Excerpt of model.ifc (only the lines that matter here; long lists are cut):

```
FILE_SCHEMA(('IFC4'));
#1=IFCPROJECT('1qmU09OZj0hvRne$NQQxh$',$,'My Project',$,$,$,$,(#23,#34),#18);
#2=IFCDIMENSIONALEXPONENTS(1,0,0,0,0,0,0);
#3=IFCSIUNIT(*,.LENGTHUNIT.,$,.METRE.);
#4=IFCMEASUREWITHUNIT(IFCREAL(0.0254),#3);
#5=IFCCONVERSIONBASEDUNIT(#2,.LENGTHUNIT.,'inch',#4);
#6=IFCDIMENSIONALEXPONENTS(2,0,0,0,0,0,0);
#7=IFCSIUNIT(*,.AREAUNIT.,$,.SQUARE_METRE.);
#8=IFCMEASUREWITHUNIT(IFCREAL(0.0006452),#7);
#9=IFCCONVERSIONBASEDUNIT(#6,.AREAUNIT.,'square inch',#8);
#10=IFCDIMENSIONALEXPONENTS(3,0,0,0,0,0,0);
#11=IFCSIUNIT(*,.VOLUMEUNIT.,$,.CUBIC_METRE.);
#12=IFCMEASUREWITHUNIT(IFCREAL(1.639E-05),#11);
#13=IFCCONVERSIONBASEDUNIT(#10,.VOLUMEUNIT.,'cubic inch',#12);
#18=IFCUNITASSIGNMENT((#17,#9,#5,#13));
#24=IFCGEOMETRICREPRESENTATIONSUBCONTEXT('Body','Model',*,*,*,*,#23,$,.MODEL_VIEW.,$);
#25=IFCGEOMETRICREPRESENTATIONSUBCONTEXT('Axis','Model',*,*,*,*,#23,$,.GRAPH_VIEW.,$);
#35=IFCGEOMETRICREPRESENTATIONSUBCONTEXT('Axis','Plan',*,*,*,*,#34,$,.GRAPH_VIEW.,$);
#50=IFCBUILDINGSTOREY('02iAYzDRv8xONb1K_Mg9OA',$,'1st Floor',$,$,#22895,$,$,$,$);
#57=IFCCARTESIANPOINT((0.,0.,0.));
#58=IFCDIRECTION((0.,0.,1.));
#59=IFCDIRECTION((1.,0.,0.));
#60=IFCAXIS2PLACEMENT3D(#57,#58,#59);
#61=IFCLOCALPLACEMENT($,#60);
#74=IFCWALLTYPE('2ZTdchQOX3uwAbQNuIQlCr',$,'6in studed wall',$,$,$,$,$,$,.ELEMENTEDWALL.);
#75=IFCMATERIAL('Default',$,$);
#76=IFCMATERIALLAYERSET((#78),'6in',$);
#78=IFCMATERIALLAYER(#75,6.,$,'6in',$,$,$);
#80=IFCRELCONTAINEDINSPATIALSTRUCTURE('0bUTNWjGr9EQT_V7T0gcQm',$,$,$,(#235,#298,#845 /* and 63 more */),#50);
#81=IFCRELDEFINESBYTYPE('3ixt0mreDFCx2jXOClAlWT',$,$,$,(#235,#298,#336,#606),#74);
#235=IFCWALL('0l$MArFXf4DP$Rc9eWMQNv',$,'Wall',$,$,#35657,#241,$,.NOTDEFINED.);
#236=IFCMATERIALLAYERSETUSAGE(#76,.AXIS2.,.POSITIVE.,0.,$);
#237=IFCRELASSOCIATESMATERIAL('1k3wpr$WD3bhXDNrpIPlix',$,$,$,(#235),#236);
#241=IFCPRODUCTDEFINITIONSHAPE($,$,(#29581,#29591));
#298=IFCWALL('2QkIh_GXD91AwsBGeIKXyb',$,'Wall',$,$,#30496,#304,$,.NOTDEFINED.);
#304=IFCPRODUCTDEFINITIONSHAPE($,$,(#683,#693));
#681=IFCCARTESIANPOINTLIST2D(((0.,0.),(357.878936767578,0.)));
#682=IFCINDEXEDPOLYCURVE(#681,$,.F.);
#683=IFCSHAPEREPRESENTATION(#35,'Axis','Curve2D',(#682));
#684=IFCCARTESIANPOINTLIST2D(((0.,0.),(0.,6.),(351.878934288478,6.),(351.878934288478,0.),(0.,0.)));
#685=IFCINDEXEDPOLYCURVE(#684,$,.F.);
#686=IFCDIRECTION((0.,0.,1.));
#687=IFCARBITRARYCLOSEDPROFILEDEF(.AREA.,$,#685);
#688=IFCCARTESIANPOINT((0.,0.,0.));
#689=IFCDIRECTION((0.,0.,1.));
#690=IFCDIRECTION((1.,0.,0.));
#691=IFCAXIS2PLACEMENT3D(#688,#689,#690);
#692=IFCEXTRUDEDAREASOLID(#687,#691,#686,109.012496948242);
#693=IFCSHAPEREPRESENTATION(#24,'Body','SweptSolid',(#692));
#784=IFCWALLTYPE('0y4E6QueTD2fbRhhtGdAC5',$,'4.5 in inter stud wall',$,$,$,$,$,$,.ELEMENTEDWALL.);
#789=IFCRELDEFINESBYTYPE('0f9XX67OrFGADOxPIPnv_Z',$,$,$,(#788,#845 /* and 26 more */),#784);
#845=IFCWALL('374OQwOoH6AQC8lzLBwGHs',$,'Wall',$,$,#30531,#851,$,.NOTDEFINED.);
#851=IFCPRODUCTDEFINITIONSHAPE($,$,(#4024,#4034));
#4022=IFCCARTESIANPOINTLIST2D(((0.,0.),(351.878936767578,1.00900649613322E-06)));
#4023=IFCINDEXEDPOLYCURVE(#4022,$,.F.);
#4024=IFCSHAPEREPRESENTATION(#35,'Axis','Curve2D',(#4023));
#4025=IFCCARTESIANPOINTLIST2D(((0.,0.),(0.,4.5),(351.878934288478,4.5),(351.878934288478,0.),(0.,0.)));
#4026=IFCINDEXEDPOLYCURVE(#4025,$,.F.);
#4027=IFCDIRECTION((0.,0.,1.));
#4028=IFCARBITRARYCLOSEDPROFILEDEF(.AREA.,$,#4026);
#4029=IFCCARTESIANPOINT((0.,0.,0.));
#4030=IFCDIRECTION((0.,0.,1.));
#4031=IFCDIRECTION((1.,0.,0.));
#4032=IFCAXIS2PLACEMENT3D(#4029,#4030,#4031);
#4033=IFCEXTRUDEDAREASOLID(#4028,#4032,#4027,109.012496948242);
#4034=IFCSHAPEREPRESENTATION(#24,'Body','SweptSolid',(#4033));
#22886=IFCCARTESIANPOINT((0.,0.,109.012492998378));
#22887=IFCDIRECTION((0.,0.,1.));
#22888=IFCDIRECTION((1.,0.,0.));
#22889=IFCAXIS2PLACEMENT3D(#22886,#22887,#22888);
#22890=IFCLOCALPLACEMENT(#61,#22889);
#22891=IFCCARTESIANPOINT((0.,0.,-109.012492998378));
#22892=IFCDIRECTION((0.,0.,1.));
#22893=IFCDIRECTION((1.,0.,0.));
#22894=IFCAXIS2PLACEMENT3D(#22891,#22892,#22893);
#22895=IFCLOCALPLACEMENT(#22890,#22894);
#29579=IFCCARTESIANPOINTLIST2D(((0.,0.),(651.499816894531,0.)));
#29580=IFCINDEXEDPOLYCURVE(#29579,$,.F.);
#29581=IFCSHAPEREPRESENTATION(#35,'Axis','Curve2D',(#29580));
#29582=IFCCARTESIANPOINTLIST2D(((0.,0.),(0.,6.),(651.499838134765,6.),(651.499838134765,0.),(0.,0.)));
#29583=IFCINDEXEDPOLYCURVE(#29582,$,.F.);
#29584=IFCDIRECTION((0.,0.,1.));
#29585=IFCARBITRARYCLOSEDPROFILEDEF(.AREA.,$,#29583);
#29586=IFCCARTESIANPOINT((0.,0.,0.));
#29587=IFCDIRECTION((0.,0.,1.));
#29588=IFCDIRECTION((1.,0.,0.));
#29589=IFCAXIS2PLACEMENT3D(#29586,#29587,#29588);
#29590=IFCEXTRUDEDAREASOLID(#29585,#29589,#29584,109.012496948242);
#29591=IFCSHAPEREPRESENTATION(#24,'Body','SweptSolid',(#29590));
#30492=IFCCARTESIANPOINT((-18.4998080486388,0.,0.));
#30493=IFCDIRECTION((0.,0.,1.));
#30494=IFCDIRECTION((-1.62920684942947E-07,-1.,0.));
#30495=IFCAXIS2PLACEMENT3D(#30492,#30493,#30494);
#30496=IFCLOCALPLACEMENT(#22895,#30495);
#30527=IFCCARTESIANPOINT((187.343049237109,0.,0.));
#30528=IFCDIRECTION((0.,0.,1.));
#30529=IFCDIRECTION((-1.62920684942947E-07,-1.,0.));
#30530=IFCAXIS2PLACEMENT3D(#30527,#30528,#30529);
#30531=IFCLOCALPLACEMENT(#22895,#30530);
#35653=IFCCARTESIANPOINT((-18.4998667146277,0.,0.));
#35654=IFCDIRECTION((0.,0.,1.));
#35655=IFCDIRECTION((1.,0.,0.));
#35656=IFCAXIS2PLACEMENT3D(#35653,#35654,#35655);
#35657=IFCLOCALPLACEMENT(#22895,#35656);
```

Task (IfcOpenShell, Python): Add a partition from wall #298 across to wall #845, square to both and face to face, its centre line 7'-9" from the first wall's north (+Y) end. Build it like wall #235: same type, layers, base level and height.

```python
import numpy as np
import ifcopenshell
import ifcopenshell.api.geometry
import ifcopenshell.api.material
import ifcopenshell.api.pset
import ifcopenshell.api.root
import ifcopenshell.api.spatial
import ifcopenshell.api.type
import ifcopenshell.geom
import ifcopenshell.util.element
import ifcopenshell.util.placement
import ifcopenshell.util.representation
import ifcopenshell.util.shape
import ifcopenshell.util.unit

model = ifcopenshell.open("model.ifc")
unit_scale = ifcopenshell.util.unit.calculate_unit_scale(model)
settings = ifcopenshell.geom.settings()
settings.set("use-world-coords", True)

start_wall = model.by_guid("2QkIh_GXD91AwsBGeIKXyb")
end_wall = model.by_id(845)
like = model.by_guid("0l$MArFXf4DP$Rc9eWMQNv")
matrix = ifcopenshell.util.placement.get_local_placement(start_wall.ObjectPlacement)
matrix[:3, 3] *= unit_scale


def extent(element):
    """Bounding box in the first wall's axes, in metres."""
    shape = ifcopenshell.geom.create_shape(settings, element)
    points = (ifcopenshell.util.shape.get_vertices(shape.geometry) - matrix[:3, 3]) @ matrix[:3, :3]
    return points.min(axis=0), points.max(axis=0)


y_start = extent(start_wall)[1][1]
y_end = extent(end_wall)[0][1]
like_min, like_max = extent(like)
length, height = float(abs(y_end - y_start)), float(like_max[2] - like_min[2])
layer_set = ifcopenshell.util.element.get_material(like, should_skip_usage=True)
thickness = sum(layer.LayerThickness for layer in layer_set.MaterialLayers) * unit_scale

wall = ifcopenshell.api.root.create_entity(model, ifc_class="IfcWall", name="New partition")
storey = ifcopenshell.util.element.get_container(like)
ifcopenshell.api.spatial.assign_container(model, products=[wall], relating_structure=storey)
ifcopenshell.api.type.assign_type(
    model, related_objects=[wall], relating_type=ifcopenshell.util.element.get_type(like), should_map_representations=False
)
rel = ifcopenshell.api.material.assign_material(
    model, products=[wall], type="IfcMaterialLayerSetUsage", material=layer_set
)
rel.RelatingMaterial.OffsetFromReferenceLine = -thickness / 2 / unit_scale
pset = ifcopenshell.api.pset.add_pset(model, product=wall, name="Pset_WallCommon")
ifcopenshell.api.pset.edit_pset(model, pset=pset, properties={"IsExternal": False, "LoadBearing": False})

# The axis runs down the middle of the wall.
axis = ifcopenshell.api.geometry.add_axis_representation(
    model, context=ifcopenshell.util.representation.get_context(model, "Model", "Axis"), axis=[(0.0, 0.0), (length, 0.0)]
)
body = ifcopenshell.api.geometry.add_wall_representation(
    model,
    context=ifcopenshell.util.representation.get_context(model, "Model", "Body", "MODEL_VIEW"),
    length=length,
    height=height,
    thickness=thickness,
    offset=-thickness / 2,
)
for representation in (axis, body):
    ifcopenshell.api.geometry.assign_representation(model, product=wall, representation=representation)

placement = matrix @ ifcopenshell.util.placement.rotation(90, "Z")
placement[:, 3] = matrix @ np.array([extent(start_wall)[0][0] + 2.3622, y_start, like_min[2], 1.0])
ifcopenshell.api.geometry.edit_object_placement(model, product=wall, matrix=placement)

print(f"partition {length:.3f} m long, {height:.3f} m high, {thickness:.3f} m thick")

model.write("model_updated.ifc")
```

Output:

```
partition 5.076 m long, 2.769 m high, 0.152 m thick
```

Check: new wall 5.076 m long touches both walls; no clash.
